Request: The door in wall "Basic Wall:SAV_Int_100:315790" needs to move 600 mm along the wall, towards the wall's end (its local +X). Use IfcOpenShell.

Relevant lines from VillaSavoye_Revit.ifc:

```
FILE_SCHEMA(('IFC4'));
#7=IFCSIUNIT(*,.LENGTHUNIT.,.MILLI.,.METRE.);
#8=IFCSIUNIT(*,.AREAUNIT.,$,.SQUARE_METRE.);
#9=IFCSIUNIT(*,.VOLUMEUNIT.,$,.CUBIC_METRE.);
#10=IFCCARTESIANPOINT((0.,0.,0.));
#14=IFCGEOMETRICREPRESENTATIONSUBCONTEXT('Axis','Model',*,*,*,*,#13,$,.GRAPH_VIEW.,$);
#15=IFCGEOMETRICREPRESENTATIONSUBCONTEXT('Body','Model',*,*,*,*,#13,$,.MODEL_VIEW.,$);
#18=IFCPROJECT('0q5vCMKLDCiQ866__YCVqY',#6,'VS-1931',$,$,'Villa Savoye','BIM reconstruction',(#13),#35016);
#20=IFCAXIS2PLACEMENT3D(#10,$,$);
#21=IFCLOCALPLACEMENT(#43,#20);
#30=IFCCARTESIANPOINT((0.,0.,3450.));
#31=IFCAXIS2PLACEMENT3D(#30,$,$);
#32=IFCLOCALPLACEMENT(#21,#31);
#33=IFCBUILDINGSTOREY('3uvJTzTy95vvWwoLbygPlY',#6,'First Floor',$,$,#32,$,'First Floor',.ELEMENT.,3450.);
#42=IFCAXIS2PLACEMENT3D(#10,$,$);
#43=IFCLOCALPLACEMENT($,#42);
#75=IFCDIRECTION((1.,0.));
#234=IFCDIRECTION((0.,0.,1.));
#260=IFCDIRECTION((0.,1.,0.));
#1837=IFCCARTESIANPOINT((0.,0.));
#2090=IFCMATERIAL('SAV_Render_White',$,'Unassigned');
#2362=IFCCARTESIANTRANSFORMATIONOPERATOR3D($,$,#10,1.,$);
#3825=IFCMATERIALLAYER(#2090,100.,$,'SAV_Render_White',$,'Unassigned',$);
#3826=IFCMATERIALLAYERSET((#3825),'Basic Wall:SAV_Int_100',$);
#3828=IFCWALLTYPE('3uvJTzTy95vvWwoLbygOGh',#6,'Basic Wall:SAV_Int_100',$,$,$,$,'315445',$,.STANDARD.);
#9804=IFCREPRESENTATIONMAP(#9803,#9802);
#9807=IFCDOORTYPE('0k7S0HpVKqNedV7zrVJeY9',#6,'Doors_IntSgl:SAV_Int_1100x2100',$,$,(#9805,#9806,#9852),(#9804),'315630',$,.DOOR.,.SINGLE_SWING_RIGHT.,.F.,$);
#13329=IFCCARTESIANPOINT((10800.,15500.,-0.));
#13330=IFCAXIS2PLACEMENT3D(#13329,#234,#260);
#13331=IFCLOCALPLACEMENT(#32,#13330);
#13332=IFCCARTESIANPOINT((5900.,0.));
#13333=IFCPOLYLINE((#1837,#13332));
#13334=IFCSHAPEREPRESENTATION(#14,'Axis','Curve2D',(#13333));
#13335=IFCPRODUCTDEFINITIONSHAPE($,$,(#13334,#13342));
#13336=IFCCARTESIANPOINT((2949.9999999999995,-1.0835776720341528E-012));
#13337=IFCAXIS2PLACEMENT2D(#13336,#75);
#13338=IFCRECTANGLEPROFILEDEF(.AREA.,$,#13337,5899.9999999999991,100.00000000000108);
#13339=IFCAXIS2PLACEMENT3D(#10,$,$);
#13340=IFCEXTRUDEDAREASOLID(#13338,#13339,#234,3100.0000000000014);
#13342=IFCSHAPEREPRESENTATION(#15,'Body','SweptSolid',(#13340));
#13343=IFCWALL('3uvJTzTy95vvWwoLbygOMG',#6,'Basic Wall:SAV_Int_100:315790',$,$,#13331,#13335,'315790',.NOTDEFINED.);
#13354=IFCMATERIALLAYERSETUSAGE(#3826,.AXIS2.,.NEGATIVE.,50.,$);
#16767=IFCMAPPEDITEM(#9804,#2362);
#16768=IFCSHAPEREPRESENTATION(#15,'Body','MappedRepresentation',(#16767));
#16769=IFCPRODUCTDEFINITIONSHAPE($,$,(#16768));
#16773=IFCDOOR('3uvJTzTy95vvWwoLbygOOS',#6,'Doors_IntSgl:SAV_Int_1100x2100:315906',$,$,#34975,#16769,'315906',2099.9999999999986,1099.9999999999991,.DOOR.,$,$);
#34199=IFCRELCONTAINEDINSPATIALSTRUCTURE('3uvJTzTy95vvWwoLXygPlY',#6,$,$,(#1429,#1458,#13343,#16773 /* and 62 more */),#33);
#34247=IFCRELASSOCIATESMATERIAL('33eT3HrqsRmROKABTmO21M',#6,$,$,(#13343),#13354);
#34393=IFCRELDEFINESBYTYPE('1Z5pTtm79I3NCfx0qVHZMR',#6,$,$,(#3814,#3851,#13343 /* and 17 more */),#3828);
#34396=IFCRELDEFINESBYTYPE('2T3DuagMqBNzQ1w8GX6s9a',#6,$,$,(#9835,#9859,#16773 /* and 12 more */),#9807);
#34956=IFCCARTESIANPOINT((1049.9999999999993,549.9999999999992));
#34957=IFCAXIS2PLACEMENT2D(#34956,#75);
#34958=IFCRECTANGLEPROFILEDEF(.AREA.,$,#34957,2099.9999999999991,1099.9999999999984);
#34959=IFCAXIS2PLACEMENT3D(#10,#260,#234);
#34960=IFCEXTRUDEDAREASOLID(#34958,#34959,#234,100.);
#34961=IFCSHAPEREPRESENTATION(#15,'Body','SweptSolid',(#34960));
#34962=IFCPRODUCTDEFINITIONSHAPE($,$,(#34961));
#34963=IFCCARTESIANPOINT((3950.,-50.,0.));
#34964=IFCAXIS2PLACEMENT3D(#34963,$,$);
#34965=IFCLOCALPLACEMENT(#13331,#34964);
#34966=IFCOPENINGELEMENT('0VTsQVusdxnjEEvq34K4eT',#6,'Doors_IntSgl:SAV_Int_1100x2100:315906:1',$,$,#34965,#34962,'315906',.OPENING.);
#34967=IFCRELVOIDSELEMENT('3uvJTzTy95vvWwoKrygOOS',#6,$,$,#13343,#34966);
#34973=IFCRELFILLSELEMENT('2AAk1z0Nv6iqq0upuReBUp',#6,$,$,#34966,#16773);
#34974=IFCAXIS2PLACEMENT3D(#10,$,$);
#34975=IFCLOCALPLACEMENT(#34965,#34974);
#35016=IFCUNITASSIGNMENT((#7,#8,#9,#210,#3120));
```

```python
import ifcopenshell
import ifcopenshell.api.geometry
import ifcopenshell.util.placement

model = ifcopenshell.open("VillaSavoye_Revit.ifc")

door = model.by_guid("3uvJTzTy95vvWwoLbygOOS")
opening = door.FillsVoids[0].RelatingOpeningElement
wall = opening.VoidsElements[0].RelatingBuildingElement

wall_matrix = ifcopenshell.util.placement.get_local_placement(wall.ObjectPlacement)
shift = wall_matrix[:3, 0] * 600.0
before = ifcopenshell.util.placement.get_local_placement(door.ObjectPlacement)[:3, 3].copy()

# The door is placed relative to its opening, so it follows when the opening moves.
matrix = ifcopenshell.util.placement.get_local_placement(opening.ObjectPlacement)
matrix[:3, 3] += shift
ifcopenshell.api.geometry.edit_object_placement(
    model, product=opening, matrix=matrix, is_si=False, should_transform_children=True
)

after = ifcopenshell.util.placement.get_local_placement(door.ObjectPlacement)[:3, 3]
print("door moved by", (after - before).round(3) + 0.0)

model.write("VillaSavoye_Revit_edited.ifc")
```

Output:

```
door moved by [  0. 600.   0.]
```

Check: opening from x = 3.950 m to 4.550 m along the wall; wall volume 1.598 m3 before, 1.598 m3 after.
